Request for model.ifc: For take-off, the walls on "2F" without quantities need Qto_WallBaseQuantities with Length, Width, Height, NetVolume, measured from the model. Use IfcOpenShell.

First a look at what the model holds.

```python
import ifcopenshell
import ifcopenshell.util.element
import ifcopenshell.util.unit

model = ifcopenshell.open("model.ifc")
print(model.schema)
for unit_type in ("LENGTHUNIT", "AREAUNIT", "VOLUMEUNIT"):
    print(unit_type, ifcopenshell.util.unit.calculate_unit_scale(model, unit_type))
storey = next(s for s in model.by_type("IfcBuildingStorey") if s.Name == "2F")
walls = [e for e in ifcopenshell.util.element.get_decomposition(storey) if e.is_a("IfcWall")]
for e in sorted(walls, key=lambda e: e.id()):
    print(e.id(), e.is_a(), e.Name, list(ifcopenshell.util.element.get_psets(e, qtos_only=True)), sep=" | ")
```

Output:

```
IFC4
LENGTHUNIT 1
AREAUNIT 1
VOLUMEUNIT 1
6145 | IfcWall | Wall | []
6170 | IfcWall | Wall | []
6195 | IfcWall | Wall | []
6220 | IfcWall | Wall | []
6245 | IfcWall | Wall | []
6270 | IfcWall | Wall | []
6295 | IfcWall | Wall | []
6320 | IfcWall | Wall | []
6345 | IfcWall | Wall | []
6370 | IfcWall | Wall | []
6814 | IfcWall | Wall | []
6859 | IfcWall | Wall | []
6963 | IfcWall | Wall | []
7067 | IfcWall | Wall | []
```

```python
import ifcopenshell
import ifcopenshell.api.pset
import ifcopenshell.geom
import ifcopenshell.util.element
import ifcopenshell.util.shape
import ifcopenshell.util.unit

model = ifcopenshell.open("model.ifc")
unit_scale = ifcopenshell.util.unit.calculate_unit_scale(model)
volume_scale = ifcopenshell.util.unit.calculate_unit_scale(model, "VOLUMEUNIT")
settings = ifcopenshell.geom.settings()

storey = next(s for s in model.by_type("IfcBuildingStorey") if s.Name == "2F")
walls = [e for e in ifcopenshell.util.element.get_decomposition(storey) if e.is_a("IfcWall")]

for e in sorted(walls, key=lambda e: e.id()):
    if ifcopenshell.util.element.get_psets(e, qtos_only=True, should_inherit=False):
        continue
    # Geometry comes back in metres, in the element's own axes.
    shape = ifcopenshell.geom.create_shape(settings, e)
    values = {
        "Length": ifcopenshell.util.shape.get_x(shape.geometry) / unit_scale,
        "Width": ifcopenshell.util.shape.get_y(shape.geometry) / unit_scale,
        "Height": ifcopenshell.util.shape.get_z(shape.geometry) / unit_scale,
        "NetVolume": ifcopenshell.util.shape.get_volume(shape.geometry) / volume_scale,
    }
    qto = ifcopenshell.api.pset.add_qto(model, product=e, name="Qto_WallBaseQuantities")
    ifcopenshell.api.pset.edit_qto(model, qto=qto, properties=values)
    print(e.id(), {k: round(v, 3) for k, v in values.items()})

model.write("model-out.ifc")
```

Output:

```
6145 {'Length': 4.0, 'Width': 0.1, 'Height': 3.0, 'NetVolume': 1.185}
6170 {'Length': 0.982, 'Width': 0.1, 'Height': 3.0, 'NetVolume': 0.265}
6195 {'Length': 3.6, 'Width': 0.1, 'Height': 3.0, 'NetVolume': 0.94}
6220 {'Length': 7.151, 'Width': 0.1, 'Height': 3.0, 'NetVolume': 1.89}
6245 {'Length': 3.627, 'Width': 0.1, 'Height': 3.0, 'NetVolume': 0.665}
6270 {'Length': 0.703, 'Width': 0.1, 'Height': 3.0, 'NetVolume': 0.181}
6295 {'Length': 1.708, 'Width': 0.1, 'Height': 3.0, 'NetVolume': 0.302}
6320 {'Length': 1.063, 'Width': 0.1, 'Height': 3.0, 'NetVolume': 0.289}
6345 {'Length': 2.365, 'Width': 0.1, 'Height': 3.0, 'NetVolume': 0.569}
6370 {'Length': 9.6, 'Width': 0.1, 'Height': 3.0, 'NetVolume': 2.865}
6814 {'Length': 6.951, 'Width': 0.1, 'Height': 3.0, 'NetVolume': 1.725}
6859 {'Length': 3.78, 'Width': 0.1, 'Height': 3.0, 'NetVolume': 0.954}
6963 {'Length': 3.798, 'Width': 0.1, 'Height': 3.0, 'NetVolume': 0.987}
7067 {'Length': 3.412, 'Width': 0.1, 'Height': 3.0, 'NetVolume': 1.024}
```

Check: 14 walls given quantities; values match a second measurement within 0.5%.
